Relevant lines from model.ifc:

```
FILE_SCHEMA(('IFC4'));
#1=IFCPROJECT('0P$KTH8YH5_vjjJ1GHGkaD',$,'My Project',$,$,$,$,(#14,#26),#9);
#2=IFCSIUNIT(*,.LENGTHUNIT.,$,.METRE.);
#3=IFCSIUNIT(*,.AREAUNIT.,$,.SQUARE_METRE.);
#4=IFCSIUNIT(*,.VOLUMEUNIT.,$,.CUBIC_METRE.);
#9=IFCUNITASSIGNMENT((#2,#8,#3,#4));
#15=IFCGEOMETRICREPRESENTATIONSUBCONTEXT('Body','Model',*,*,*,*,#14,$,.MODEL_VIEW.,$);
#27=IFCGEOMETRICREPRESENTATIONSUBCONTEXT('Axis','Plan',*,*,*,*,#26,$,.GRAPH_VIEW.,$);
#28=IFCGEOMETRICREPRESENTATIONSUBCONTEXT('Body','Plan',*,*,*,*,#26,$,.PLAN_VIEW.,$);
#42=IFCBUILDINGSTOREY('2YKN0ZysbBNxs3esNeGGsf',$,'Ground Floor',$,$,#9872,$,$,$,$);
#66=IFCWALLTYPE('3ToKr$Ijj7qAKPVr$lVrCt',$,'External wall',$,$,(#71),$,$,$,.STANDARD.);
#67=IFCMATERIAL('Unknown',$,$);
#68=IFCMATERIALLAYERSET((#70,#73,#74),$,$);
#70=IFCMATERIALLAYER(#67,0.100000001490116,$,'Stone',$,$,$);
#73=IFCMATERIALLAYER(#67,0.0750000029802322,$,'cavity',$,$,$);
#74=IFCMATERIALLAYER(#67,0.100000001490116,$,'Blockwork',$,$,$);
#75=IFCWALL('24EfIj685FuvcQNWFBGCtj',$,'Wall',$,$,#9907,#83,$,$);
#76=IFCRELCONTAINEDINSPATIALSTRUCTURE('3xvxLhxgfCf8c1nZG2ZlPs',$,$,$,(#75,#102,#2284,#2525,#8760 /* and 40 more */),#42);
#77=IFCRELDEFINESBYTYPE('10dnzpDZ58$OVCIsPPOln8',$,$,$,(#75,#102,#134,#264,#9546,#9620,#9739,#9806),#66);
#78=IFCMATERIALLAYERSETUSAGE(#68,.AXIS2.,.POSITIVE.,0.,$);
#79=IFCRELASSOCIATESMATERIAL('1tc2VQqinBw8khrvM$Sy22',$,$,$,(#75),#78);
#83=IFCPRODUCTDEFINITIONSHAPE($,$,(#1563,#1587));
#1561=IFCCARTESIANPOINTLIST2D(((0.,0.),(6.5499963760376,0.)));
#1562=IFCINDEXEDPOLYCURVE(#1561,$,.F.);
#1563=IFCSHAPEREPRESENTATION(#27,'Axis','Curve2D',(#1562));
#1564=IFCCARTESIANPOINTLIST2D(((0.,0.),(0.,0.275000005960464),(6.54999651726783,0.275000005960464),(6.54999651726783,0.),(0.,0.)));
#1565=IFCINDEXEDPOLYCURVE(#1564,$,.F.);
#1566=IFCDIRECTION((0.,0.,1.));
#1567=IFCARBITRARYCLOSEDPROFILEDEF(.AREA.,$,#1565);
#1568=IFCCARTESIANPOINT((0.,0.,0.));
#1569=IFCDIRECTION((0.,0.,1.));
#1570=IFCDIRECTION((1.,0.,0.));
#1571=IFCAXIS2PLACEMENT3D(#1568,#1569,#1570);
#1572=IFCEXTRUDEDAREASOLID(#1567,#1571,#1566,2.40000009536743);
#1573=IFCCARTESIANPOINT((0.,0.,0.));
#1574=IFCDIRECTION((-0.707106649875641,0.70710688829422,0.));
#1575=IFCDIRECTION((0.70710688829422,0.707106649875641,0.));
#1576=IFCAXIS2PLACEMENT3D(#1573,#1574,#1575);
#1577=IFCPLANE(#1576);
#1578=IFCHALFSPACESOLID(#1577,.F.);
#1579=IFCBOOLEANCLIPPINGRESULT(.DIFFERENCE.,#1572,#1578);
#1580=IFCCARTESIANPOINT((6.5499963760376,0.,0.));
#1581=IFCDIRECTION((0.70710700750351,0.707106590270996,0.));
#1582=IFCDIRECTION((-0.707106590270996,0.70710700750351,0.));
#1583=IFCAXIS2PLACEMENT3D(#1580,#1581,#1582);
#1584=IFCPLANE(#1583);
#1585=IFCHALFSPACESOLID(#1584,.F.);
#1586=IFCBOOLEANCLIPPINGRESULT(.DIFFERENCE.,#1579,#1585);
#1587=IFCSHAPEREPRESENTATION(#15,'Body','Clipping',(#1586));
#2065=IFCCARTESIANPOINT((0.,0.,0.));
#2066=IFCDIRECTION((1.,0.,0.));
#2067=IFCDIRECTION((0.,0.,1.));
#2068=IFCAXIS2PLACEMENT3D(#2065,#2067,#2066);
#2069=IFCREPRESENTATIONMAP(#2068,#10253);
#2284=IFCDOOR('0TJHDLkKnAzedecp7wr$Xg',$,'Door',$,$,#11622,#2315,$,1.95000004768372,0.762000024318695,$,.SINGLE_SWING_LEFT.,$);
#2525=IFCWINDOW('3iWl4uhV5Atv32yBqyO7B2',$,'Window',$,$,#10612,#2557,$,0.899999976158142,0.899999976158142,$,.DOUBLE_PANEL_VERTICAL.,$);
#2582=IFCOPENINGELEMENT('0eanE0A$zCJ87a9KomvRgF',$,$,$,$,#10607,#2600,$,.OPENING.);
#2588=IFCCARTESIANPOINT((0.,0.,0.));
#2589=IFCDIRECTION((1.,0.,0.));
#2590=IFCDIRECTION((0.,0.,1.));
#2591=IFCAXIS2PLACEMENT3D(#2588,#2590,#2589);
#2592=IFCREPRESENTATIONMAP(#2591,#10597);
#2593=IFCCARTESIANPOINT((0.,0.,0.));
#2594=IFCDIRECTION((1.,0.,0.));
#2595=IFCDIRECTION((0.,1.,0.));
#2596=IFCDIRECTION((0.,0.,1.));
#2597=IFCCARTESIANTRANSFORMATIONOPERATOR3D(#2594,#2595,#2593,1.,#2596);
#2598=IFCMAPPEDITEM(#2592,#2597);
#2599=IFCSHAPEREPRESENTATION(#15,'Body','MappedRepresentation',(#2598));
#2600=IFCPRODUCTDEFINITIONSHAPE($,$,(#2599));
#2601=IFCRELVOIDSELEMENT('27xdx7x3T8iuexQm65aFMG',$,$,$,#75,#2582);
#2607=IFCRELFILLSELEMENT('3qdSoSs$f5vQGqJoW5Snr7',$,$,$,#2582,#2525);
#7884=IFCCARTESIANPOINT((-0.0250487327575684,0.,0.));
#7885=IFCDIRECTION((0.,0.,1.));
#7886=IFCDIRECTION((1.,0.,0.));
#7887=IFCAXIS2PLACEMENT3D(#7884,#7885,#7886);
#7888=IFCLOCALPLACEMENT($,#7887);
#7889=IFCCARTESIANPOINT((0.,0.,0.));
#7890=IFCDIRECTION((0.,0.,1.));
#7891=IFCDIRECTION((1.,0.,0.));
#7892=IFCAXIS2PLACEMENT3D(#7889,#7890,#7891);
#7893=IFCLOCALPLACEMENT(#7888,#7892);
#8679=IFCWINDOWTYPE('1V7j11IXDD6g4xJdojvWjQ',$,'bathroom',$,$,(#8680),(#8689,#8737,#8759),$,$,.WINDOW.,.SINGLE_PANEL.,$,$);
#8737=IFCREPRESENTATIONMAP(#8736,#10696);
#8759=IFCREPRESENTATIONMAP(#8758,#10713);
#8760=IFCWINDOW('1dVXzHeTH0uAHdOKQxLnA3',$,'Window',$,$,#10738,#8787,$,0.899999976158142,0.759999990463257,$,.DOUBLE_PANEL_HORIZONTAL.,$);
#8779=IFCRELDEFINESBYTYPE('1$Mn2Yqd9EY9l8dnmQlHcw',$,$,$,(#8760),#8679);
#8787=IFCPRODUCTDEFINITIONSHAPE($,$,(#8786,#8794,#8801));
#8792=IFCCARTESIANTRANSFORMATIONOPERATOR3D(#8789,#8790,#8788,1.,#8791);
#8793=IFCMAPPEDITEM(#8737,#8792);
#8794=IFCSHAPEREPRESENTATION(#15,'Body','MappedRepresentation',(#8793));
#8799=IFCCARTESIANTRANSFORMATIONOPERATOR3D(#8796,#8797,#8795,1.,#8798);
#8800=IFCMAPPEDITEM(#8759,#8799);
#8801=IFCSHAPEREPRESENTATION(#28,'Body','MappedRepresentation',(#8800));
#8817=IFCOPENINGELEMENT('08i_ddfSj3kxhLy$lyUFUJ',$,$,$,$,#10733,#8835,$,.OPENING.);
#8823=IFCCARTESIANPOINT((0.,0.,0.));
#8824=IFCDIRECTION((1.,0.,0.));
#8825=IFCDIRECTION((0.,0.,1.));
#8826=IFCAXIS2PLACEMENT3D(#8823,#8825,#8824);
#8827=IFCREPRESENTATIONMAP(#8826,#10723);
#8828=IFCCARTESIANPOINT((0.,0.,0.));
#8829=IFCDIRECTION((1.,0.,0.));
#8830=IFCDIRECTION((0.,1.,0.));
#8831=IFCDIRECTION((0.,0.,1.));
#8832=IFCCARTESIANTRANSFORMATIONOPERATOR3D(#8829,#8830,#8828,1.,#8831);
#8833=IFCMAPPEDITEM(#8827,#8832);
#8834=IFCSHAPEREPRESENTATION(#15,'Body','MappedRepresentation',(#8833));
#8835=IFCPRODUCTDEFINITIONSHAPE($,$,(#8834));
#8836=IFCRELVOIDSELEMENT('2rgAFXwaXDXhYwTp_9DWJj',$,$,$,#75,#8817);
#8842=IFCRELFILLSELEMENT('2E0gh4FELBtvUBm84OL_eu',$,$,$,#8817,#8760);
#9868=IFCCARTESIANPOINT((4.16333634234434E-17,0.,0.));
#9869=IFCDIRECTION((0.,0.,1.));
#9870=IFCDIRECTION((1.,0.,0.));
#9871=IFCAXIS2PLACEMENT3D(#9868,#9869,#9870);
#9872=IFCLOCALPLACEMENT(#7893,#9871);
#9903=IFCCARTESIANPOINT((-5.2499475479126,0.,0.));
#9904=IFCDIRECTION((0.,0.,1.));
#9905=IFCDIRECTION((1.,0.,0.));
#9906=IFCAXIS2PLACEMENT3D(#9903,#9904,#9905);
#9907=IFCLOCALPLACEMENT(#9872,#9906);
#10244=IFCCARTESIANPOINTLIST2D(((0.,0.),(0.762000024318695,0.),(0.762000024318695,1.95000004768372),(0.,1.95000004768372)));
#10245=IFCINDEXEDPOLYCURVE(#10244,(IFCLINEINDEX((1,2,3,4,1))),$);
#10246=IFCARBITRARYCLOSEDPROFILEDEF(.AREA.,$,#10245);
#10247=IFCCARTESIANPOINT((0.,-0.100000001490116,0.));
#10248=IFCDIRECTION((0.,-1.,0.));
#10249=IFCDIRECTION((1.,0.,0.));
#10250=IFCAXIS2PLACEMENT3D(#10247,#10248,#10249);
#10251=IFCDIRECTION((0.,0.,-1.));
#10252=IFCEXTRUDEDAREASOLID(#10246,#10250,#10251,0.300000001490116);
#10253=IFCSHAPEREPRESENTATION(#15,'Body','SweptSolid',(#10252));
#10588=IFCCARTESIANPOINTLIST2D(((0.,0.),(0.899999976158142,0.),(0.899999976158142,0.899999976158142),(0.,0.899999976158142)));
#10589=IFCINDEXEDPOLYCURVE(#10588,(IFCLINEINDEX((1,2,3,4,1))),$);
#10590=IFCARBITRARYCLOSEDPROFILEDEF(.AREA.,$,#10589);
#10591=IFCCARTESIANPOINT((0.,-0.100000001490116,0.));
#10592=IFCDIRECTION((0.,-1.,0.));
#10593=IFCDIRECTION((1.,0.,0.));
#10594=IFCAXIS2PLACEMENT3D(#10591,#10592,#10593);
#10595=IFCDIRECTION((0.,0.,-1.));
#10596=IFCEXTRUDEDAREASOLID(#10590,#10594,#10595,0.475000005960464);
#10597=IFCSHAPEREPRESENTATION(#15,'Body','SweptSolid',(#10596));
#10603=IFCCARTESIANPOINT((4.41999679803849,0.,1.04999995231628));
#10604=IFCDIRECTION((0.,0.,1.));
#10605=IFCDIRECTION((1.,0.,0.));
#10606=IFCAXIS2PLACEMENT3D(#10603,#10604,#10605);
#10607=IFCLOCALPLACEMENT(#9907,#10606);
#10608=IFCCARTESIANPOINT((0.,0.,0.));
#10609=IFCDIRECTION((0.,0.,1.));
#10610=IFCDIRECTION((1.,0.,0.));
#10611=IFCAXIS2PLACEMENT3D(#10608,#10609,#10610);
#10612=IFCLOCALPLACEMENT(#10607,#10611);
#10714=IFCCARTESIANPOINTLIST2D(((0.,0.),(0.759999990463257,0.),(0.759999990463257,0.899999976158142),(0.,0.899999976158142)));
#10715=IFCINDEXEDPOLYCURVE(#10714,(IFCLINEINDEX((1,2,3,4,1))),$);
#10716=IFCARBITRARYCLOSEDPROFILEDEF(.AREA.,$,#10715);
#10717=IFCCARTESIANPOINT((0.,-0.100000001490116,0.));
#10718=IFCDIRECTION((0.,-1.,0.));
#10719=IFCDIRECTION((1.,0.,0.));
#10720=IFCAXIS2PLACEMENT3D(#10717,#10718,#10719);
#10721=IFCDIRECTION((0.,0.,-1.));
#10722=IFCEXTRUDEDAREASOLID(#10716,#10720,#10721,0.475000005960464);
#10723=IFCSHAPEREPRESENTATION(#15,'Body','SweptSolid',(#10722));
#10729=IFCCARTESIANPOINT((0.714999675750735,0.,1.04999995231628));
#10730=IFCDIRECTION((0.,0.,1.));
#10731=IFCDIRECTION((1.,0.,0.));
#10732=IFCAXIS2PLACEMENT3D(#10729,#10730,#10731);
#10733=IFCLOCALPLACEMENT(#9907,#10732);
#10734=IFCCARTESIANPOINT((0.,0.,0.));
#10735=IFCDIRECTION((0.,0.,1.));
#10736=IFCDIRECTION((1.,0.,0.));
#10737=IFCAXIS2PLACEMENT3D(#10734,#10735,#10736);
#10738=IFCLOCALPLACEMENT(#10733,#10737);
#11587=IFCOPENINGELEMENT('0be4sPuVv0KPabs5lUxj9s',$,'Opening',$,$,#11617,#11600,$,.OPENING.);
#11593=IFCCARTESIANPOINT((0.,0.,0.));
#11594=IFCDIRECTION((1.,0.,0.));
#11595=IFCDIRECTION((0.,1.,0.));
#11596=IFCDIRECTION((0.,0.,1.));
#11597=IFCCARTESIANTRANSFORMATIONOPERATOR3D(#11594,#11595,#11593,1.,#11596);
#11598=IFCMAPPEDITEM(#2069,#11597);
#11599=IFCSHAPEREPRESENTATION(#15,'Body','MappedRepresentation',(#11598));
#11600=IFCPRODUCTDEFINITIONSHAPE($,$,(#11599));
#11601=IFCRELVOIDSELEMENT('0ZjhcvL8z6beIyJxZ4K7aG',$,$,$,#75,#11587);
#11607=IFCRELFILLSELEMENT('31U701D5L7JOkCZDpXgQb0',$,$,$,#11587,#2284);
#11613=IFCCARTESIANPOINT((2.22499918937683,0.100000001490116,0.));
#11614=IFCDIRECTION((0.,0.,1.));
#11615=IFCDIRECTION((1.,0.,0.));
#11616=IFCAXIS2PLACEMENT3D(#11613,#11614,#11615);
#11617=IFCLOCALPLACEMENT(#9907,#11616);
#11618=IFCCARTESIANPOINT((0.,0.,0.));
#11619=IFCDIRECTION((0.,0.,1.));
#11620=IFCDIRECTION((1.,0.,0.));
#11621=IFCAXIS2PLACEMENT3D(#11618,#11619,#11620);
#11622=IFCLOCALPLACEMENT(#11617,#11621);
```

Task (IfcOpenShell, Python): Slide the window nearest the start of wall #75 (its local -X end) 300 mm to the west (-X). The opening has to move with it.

```python
import ifcopenshell
import ifcopenshell.api.geometry
import ifcopenshell.util.placement

model = ifcopenshell.open("model.ifc")

window = model.by_id(8760)
opening = window.FillsVoids[0].RelatingOpeningElement
wall = opening.VoidsElements[0].RelatingBuildingElement

wall_matrix = ifcopenshell.util.placement.get_local_placement(wall.ObjectPlacement)
shift = wall_matrix[:3, 0] * -0.3
before = ifcopenshell.util.placement.get_local_placement(window.ObjectPlacement)[:3, 3].copy()

# The window is placed relative to its opening, so it follows when the opening moves.
matrix = ifcopenshell.util.placement.get_local_placement(opening.ObjectPlacement)
matrix[:3, 3] += shift
ifcopenshell.api.geometry.edit_object_placement(
    model, product=opening, matrix=matrix, is_si=False, should_transform_children=True
)

after = ifcopenshell.util.placement.get_local_placement(window.ObjectPlacement)[:3, 3]
print("window moved by", (after - before).round(3) + 0.0)

model.write("model_rev.ifc")
```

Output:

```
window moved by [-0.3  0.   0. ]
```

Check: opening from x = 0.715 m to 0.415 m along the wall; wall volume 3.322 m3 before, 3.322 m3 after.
